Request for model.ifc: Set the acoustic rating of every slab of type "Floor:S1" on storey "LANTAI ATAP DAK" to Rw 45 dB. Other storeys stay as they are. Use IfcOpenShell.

First a look at what the model holds.

```python
import ifcopenshell
import ifcopenshell.util.element

model = ifcopenshell.open("model.ifc")
print(model.schema)
storey = next(s for s in model.by_type("IfcBuildingStorey") if s.Name == "LANTAI ATAP DAK")
slabs = [e for e in ifcopenshell.util.element.get_decomposition(storey) if e.is_a("IfcSlab")]
seen = {}
for e in slabs:
    element_type = ifcopenshell.util.element.get_type(e)
    key = (element_type.Name if element_type != e and element_type else None, ifcopenshell.util.element.get_pset(e, "Pset_SlabCommon", "AcousticRating"))
    seen[key] = seen.get(key, 0) + 1
for (name, value), count in sorted(seen.items(), key=str):
    print(count, "x", name, "|", value)
```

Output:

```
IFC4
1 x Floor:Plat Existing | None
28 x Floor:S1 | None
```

```python
import ifcopenshell
import ifcopenshell.api.pset
import ifcopenshell.util.element

model = ifcopenshell.open("model.ifc")

storey = next(s for s in model.by_type("IfcBuildingStorey") if s.Name == "LANTAI ATAP DAK")
slabs = [e for e in ifcopenshell.util.element.get_decomposition(storey) if e.is_a("IfcSlab")]

count = 0
for e in slabs:
    element_type = ifcopenshell.util.element.get_type(e)
    if element_type in (None, e) or element_type.Name != "Floor:S1":
        continue
    # add_pset returns the element's existing set when there is one.
    pset = ifcopenshell.api.pset.add_pset(model, product=e, name="Pset_SlabCommon")
    ifcopenshell.api.pset.edit_pset(model, pset=pset, properties={"AcousticRating": "Rw 45 dB"})
    count += 1

print(count, "slabs updated")

model.write("model_rev.ifc")
```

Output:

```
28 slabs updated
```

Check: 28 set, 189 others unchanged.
